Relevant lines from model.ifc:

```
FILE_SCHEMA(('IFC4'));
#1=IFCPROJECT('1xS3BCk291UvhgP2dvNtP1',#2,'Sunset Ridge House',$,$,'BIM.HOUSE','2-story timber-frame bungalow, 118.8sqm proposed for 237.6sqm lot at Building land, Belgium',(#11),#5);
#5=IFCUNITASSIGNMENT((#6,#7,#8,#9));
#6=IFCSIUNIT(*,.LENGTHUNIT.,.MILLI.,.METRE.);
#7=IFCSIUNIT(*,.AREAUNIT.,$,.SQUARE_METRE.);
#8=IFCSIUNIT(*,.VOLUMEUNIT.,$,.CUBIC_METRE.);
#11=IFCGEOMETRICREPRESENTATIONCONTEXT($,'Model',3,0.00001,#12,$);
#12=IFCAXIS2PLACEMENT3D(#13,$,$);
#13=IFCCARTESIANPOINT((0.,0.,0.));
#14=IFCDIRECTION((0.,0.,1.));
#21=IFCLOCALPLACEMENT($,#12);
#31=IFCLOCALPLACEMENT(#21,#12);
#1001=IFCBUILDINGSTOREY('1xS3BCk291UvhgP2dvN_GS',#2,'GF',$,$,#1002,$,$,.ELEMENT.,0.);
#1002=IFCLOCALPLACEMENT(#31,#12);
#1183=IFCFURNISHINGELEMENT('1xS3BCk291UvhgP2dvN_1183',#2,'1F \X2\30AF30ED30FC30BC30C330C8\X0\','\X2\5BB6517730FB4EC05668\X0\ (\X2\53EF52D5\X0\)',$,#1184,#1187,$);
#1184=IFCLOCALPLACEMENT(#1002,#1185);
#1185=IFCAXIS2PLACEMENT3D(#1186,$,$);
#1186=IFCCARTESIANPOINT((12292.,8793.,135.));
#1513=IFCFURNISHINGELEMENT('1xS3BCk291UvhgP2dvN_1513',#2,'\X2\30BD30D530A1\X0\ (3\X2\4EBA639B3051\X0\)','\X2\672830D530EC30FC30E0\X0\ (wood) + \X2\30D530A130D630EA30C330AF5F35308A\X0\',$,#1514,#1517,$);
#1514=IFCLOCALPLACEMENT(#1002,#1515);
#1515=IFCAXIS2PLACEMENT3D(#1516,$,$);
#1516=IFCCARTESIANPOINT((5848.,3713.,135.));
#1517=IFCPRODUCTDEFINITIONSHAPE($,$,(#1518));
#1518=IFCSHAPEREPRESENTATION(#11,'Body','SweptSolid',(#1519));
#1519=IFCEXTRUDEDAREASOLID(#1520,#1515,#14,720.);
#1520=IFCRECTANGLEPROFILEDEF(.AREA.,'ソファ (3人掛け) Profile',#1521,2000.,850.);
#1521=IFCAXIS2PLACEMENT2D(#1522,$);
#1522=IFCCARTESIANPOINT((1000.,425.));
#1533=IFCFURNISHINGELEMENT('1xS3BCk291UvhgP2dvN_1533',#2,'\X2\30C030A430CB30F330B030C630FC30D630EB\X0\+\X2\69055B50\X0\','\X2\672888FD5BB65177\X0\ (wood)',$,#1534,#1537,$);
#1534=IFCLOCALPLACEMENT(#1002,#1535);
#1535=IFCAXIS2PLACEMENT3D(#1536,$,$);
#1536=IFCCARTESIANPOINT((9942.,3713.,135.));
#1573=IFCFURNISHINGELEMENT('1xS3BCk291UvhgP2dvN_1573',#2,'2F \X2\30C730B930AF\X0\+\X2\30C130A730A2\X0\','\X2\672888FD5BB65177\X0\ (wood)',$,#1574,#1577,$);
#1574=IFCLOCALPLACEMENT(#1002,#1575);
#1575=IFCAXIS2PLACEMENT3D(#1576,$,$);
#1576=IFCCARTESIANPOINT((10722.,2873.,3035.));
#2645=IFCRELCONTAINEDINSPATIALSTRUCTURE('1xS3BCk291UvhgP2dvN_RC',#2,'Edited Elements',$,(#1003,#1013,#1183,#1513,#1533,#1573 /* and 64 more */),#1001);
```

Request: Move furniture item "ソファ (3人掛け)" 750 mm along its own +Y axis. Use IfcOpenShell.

```python
import ifcopenshell
import ifcopenshell.api.geometry
import ifcopenshell.util.placement
import ifcopenshell.util.unit

model = ifcopenshell.open("model.ifc")
unit_scale = ifcopenshell.util.unit.calculate_unit_scale(model)

item = model.by_id(1513)
matrix = ifcopenshell.util.placement.get_local_placement(item.ObjectPlacement)
matrix[:3, 3] += matrix[:3, 1] * 0.75 / unit_scale
ifcopenshell.api.geometry.edit_object_placement(model, product=item, matrix=matrix, is_si=False)

print(ifcopenshell.util.placement.get_local_placement(item.ObjectPlacement).round(3) + 0.0)

model.write("model_v2.ifc")
```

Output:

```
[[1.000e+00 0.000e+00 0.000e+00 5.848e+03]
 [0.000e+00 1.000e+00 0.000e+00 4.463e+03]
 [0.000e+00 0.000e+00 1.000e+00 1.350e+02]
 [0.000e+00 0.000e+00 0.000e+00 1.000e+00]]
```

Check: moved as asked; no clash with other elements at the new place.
